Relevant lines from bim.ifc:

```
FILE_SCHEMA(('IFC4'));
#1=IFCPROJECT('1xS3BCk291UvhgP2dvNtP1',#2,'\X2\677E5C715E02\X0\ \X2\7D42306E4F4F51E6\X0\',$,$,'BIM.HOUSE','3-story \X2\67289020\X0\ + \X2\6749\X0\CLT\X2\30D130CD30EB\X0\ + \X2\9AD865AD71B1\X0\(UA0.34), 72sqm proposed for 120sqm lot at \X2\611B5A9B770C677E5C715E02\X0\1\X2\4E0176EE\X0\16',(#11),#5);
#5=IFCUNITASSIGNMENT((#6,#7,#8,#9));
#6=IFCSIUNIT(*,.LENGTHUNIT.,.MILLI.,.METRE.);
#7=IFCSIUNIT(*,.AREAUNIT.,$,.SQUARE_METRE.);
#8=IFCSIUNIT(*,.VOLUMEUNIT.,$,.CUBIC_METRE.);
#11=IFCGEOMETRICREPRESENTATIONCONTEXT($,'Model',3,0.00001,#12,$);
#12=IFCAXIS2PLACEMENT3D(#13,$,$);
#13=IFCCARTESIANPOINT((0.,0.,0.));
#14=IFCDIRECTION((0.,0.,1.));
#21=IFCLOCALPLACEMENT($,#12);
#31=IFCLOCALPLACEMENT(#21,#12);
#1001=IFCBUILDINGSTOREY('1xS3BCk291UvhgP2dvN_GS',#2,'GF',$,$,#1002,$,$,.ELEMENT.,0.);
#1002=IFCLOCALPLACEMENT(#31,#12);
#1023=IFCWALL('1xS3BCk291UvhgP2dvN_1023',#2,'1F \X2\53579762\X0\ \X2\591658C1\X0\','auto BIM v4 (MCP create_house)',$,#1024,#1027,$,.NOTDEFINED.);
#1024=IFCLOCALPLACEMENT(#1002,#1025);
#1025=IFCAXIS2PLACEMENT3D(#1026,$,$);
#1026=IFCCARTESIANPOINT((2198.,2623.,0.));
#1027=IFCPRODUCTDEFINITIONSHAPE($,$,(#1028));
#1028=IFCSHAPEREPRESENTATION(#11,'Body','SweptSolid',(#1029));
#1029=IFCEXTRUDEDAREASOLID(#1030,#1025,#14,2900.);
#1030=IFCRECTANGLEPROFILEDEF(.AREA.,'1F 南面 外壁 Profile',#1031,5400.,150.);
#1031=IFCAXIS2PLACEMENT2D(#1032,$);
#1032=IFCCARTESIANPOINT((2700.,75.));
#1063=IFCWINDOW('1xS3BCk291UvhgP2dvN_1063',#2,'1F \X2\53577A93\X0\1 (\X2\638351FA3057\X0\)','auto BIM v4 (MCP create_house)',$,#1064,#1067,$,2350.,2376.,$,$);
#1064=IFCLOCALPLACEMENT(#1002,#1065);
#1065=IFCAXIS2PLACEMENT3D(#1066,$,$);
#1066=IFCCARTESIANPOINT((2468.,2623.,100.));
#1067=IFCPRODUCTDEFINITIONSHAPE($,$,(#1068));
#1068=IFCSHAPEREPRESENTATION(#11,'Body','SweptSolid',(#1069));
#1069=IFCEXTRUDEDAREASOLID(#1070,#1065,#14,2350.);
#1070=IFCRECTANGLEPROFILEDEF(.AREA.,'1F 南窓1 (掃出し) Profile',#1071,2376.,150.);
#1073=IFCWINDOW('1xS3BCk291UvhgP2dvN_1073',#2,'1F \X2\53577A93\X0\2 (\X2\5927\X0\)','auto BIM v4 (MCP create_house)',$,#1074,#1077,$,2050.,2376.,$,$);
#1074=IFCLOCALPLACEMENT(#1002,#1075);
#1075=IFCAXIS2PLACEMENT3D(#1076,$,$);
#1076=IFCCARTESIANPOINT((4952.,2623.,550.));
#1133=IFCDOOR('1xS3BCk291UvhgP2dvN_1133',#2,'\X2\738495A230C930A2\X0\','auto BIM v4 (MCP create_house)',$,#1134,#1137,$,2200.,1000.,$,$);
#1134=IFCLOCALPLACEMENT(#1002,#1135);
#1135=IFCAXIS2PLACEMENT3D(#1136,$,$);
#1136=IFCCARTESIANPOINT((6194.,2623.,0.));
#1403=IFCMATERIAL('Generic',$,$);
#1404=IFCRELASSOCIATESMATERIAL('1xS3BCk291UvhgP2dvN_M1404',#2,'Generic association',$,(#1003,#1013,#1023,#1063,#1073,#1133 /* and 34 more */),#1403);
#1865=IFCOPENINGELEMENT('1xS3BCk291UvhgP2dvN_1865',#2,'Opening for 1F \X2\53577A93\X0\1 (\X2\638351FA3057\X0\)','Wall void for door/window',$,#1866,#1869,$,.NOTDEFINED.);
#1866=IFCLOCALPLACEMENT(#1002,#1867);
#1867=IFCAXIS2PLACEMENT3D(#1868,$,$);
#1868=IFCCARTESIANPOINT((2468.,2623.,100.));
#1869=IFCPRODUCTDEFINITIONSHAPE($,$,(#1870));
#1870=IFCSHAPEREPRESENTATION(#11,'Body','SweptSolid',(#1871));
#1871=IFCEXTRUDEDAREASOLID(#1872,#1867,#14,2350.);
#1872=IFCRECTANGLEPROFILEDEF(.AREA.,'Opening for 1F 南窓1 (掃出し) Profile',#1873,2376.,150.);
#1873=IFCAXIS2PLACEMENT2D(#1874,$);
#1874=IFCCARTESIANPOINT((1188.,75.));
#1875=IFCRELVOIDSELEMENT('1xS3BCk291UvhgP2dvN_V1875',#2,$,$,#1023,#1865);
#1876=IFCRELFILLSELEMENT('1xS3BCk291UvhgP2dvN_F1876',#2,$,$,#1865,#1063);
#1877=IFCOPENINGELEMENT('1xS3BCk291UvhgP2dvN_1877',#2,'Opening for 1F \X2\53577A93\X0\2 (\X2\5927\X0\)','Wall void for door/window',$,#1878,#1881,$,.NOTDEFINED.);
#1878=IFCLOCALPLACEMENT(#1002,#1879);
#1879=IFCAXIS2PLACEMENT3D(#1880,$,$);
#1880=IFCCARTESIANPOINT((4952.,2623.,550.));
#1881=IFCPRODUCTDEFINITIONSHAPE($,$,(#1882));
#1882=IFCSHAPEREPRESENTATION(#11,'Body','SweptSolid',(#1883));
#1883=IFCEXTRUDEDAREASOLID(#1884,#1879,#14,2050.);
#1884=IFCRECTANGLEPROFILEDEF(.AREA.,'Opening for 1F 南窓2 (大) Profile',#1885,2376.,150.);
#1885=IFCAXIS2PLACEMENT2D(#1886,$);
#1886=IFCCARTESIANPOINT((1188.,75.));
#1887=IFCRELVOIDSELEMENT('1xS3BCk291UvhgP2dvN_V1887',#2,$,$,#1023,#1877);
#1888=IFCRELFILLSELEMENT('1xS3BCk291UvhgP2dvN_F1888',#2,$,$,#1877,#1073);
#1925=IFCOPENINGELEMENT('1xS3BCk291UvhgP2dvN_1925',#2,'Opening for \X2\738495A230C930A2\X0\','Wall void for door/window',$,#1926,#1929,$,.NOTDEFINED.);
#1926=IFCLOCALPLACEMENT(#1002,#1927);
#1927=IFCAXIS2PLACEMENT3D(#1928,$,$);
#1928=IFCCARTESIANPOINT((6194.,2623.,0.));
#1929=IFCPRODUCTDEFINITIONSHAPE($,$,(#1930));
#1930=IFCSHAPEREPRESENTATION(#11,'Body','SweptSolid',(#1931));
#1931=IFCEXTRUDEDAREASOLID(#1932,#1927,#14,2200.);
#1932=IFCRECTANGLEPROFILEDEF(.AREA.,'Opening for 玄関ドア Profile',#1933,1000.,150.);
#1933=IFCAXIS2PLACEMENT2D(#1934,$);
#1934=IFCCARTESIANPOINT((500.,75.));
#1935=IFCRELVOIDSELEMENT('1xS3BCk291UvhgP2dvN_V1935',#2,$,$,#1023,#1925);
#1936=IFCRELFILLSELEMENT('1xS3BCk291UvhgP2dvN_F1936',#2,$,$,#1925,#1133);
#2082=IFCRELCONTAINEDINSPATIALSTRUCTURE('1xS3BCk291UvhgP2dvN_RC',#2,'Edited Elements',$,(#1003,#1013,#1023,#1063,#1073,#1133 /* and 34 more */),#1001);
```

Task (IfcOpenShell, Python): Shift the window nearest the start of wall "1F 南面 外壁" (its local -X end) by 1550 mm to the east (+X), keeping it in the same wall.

```python
import ifcopenshell
import ifcopenshell.api.geometry
import ifcopenshell.util.placement
import ifcopenshell.util.unit

model = ifcopenshell.open("bim.ifc")
unit_scale = ifcopenshell.util.unit.calculate_unit_scale(model)

window = model.by_guid("1xS3BCk291UvhgP2dvN_1063")
opening = window.FillsVoids[0].RelatingOpeningElement
wall = opening.VoidsElements[0].RelatingBuildingElement

wall_matrix = ifcopenshell.util.placement.get_local_placement(wall.ObjectPlacement)
shift = wall_matrix[:3, 0] * 1.55 / unit_scale
before = ifcopenshell.util.placement.get_local_placement(window.ObjectPlacement)[:3, 3].copy()

# The window is not placed relative to its opening, so move both.
for product in (opening, window):
    matrix = ifcopenshell.util.placement.get_local_placement(product.ObjectPlacement)
    matrix[:3, 3] += shift
    ifcopenshell.api.geometry.edit_object_placement(model, product=product, matrix=matrix, is_si=False)

after = ifcopenshell.util.placement.get_local_placement(window.ObjectPlacement)[:3, 3]
print("window moved by", (after - before).round(3) + 0.0)

model.write("bim_v2.ifc")
```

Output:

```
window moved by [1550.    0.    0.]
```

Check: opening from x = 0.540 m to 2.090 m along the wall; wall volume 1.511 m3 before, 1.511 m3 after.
